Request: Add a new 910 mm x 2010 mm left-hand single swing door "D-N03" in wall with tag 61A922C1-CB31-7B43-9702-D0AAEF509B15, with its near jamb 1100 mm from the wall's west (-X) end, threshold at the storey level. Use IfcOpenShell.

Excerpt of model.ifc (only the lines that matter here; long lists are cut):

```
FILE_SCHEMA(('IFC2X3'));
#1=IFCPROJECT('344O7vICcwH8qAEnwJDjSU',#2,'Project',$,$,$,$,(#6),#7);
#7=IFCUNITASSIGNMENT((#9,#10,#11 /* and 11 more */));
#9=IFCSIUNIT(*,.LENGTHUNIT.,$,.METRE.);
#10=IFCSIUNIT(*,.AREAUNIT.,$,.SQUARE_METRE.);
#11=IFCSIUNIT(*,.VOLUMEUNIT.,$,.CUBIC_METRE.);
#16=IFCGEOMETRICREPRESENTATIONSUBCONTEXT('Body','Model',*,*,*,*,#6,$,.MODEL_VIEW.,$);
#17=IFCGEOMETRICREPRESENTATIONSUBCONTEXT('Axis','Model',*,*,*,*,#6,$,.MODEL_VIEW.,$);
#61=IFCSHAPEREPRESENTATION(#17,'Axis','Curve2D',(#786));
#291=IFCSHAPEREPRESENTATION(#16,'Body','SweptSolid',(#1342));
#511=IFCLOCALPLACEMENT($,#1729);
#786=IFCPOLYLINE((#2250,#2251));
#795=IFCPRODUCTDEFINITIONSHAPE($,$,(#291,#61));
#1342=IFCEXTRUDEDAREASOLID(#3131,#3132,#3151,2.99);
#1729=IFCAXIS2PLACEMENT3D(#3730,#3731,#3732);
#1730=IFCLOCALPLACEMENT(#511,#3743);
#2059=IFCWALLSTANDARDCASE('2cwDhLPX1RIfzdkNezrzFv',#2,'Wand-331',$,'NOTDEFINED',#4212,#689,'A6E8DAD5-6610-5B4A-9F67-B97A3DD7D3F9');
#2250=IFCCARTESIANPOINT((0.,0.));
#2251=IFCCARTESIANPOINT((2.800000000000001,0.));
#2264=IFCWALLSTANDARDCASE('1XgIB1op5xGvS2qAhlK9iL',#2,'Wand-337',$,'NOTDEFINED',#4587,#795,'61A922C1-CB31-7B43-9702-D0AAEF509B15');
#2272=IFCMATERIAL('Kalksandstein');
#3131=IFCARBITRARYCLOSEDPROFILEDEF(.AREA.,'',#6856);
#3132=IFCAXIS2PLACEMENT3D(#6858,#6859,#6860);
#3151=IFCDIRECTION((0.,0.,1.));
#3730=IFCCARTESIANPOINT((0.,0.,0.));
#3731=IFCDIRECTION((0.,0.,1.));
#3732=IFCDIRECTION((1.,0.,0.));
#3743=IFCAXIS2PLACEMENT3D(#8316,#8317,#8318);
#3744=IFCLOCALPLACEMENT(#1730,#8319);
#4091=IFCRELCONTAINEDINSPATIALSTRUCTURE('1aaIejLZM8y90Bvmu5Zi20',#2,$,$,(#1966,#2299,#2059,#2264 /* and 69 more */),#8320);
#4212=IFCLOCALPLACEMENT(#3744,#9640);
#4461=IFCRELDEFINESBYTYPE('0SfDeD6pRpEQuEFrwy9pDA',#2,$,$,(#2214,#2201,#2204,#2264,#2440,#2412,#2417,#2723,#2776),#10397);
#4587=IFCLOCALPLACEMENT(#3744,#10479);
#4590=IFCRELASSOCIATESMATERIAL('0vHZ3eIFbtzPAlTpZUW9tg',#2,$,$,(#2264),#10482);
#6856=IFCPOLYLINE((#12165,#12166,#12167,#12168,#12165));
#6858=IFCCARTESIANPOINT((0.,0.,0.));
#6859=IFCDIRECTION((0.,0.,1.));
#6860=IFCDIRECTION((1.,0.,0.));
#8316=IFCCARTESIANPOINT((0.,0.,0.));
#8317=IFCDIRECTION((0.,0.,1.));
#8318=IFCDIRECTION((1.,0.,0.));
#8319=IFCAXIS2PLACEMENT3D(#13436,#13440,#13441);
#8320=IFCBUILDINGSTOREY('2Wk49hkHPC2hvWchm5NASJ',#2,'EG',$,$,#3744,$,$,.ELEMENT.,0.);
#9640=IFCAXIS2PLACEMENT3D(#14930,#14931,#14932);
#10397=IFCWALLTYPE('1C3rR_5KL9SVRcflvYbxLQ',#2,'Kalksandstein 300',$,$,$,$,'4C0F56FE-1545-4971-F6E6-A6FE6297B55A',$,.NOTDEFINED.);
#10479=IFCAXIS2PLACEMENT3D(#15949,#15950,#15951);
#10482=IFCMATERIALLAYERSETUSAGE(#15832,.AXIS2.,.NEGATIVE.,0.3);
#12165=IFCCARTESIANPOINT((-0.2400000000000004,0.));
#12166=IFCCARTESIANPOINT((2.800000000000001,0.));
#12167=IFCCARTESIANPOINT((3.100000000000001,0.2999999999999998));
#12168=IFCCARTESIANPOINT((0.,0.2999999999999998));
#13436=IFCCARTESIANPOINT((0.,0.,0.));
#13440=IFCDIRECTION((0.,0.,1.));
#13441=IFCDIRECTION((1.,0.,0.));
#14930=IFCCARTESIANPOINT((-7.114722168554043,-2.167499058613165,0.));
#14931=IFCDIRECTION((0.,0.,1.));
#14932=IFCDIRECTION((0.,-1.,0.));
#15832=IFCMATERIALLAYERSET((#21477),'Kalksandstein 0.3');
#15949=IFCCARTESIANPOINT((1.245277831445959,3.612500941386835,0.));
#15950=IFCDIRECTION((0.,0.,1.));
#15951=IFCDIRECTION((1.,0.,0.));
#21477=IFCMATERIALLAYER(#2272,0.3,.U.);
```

```python
import numpy as np
import ifcopenshell
import ifcopenshell.api.feature
import ifcopenshell.api.geometry
import ifcopenshell.api.root
import ifcopenshell.api.spatial
import ifcopenshell.api.type
import ifcopenshell.geom
import ifcopenshell.util.element
import ifcopenshell.util.placement
import ifcopenshell.util.representation
import ifcopenshell.util.shape
import ifcopenshell.util.unit

model = ifcopenshell.open("model.ifc")
unit_scale = ifcopenshell.util.unit.calculate_unit_scale(model)
settings = ifcopenshell.geom.settings()


def volume(element):
    """Net volume in cubic metres, openings subtracted."""
    shape = ifcopenshell.geom.create_shape(settings, element)
    return ifcopenshell.util.shape.get_volume(shape.geometry)


wall = model.by_guid("1XgIB1op5xGvS2qAhlK9iL")
storey = ifcopenshell.util.element.get_container(wall, ifc_class="IfcBuildingStorey")
context = ifcopenshell.util.representation.get_context(model, "Model", "Body", "MODEL_VIEW")
before = volume(wall)

width, height, from_end, sill = 0.91, 2.01, 1.1, 0.0  # metres

# The wall runs along its own X axis, and the end named is its -X end.
wall_shape = ifcopenshell.geom.create_shape(settings, wall)
x, y, z = ifcopenshell.util.shape.get_vertices(wall_shape.geometry).T
start = x.min() + from_end
face, thickness = float(y.min()), float(y.max() - y.min())
wall_matrix = ifcopenshell.util.placement.get_local_placement(wall.ObjectPlacement)
level = ifcopenshell.util.placement.get_local_placement(storey.ObjectPlacement)[2, 3]


def in_wall(x, y):
    """Placement at x, y metres in the wall's axes, at sill height."""
    matrix = wall_matrix.copy()
    matrix[:, 3] = wall_matrix @ np.array([x / unit_scale, y / unit_scale, 0.0, 1.0])
    matrix[2, 3] = level + sill / unit_scale
    return matrix


# Opening: a box that overshoots both wall faces by 50 mm.
opening = ifcopenshell.api.root.create_entity(model, ifc_class="IfcOpeningElement")
box = ifcopenshell.api.geometry.add_wall_representation(
    model, context=context, length=width, height=height, thickness=thickness + 0.1
)
ifcopenshell.api.geometry.assign_representation(model, product=opening, representation=box)
ifcopenshell.api.geometry.edit_object_placement(model, product=opening, matrix=in_wall(start, face - 0.05), is_si=False)
ifcopenshell.api.feature.add_feature(model, feature=opening, element=wall)

door = ifcopenshell.api.root.create_entity(model, ifc_class="IfcDoor", name="D-N03")
door.OverallWidth, door.OverallHeight = width / unit_scale, height / unit_scale
body = ifcopenshell.api.geometry.add_door_representation(
    model,
    context=context,
    overall_width=door.OverallWidth,
    overall_height=door.OverallHeight,
    operation_type="SINGLE_SWING_LEFT",
    lining_properties={"LiningDepth": thickness / unit_scale, "ThresholdDepth": thickness / unit_scale},
)
ifcopenshell.api.geometry.assign_representation(model, product=door, representation=body)
ifcopenshell.api.spatial.assign_container(model, products=[door], relating_structure=storey)
fills = ifcopenshell.api.feature.add_filling(model, opening=opening, element=door)
fills.OwnerHistory = door.OwnerHistory  # required in IFC2X3

# IFC2X3 keeps the operation on the door style.
style = ifcopenshell.api.root.create_entity(model, ifc_class="IfcDoorStyle", name="D-N03")
style.OperationType, style.ConstructionType = "SINGLE_SWING_LEFT", "NOTDEFINED"
style.ParameterTakesPrecedence = style.Sizeable = False
ifcopenshell.api.type.assign_type(model, related_objects=[door], relating_type=style)

# The lining spans the wall, so the door starts at the wall face.
ifcopenshell.api.geometry.edit_object_placement(model, product=door, matrix=in_wall(start, face), is_si=False)

after = volume(wall)

print(f"wall volume {before:.3f} -> {after:.3f} m3")

model.write("model_rev.ifc")
```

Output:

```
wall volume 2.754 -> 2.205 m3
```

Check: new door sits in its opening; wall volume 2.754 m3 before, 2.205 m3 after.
